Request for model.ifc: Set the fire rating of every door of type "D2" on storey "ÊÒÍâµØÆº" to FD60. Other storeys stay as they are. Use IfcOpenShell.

First a look at what the model holds.

```python
import ifcopenshell
import ifcopenshell.util.element

model = ifcopenshell.open("model.ifc")
print(model.schema)
storey = next(s for s in model.by_type("IfcBuildingStorey") if s.Name == "ÊÒÍâµØÆº")
doors = [e for e in ifcopenshell.util.element.get_decomposition(storey) if e.is_a("IfcDoor")]
seen = {}
for e in doors:
    element_type = ifcopenshell.util.element.get_type(e)
    key = (element_type.Name if element_type != e and element_type else None, ifcopenshell.util.element.get_pset(e, "Pset_DoorCommon", "FireRating"))
    seen[key] = seen.get(key, 0) + 1
for (name, value), count in sorted(seen.items(), key=str):
    print(count, "x", name, "|", value)
```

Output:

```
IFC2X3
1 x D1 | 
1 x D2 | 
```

```python
import ifcopenshell
import ifcopenshell.api.pset
import ifcopenshell.util.element

model = ifcopenshell.open("model.ifc")

storey = next(s for s in model.by_type("IfcBuildingStorey") if s.Name == "ÊÒÍâµØÆº")
doors = [e for e in ifcopenshell.util.element.get_decomposition(storey) if e.is_a("IfcDoor")]

count = 0
for e in doors:
    element_type = ifcopenshell.util.element.get_type(e)
    if element_type in (None, e) or element_type.Name != "D2":
        continue
    # add_pset returns the element's existing set when there is one.
    pset = ifcopenshell.api.pset.add_pset(model, product=e, name="Pset_DoorCommon")
    ifcopenshell.api.pset.edit_pset(model, pset=pset, properties={"FireRating": "FD60"})
    count += 1

print(count, "doors updated")

model.write("model-out.ifc")
```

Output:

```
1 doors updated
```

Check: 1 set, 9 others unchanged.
